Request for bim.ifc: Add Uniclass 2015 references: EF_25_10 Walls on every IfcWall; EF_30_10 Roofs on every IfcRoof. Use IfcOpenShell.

First a look at what the model holds.

```python
import ifcopenshell

model = ifcopenshell.open("bim.ifc")
print(model.schema)
print("classifications:", [c.Name for c in model.by_type("IfcClassification")])
for ifc_class in ("IfcDoor", "IfcRoof", "IfcStair", "IfcWall", "IfcWindow"):
    print(ifc_class, len(model.by_type(ifc_class)))
```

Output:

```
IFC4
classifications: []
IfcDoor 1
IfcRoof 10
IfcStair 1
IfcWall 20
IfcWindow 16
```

```python
import ifcopenshell
import ifcopenshell.api.classification

model = ifcopenshell.open("bim.ifc")

system = ifcopenshell.api.classification.add_classification(model, classification="Uniclass 2015")

codes = {
    "IfcWall": ("EF_25_10", "Walls"),
    "IfcRoof": ("EF_30_10", "Roofs"),
}
for ifc_class, (code, name) in codes.items():
    products = model.by_type(ifc_class)
    ifcopenshell.api.classification.add_reference(
        model, products=products, classification=system, identification=code, name=name
    )
    print(code, len(products))

model.write("bim_updated.ifc")
```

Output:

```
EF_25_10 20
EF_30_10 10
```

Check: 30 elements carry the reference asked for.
